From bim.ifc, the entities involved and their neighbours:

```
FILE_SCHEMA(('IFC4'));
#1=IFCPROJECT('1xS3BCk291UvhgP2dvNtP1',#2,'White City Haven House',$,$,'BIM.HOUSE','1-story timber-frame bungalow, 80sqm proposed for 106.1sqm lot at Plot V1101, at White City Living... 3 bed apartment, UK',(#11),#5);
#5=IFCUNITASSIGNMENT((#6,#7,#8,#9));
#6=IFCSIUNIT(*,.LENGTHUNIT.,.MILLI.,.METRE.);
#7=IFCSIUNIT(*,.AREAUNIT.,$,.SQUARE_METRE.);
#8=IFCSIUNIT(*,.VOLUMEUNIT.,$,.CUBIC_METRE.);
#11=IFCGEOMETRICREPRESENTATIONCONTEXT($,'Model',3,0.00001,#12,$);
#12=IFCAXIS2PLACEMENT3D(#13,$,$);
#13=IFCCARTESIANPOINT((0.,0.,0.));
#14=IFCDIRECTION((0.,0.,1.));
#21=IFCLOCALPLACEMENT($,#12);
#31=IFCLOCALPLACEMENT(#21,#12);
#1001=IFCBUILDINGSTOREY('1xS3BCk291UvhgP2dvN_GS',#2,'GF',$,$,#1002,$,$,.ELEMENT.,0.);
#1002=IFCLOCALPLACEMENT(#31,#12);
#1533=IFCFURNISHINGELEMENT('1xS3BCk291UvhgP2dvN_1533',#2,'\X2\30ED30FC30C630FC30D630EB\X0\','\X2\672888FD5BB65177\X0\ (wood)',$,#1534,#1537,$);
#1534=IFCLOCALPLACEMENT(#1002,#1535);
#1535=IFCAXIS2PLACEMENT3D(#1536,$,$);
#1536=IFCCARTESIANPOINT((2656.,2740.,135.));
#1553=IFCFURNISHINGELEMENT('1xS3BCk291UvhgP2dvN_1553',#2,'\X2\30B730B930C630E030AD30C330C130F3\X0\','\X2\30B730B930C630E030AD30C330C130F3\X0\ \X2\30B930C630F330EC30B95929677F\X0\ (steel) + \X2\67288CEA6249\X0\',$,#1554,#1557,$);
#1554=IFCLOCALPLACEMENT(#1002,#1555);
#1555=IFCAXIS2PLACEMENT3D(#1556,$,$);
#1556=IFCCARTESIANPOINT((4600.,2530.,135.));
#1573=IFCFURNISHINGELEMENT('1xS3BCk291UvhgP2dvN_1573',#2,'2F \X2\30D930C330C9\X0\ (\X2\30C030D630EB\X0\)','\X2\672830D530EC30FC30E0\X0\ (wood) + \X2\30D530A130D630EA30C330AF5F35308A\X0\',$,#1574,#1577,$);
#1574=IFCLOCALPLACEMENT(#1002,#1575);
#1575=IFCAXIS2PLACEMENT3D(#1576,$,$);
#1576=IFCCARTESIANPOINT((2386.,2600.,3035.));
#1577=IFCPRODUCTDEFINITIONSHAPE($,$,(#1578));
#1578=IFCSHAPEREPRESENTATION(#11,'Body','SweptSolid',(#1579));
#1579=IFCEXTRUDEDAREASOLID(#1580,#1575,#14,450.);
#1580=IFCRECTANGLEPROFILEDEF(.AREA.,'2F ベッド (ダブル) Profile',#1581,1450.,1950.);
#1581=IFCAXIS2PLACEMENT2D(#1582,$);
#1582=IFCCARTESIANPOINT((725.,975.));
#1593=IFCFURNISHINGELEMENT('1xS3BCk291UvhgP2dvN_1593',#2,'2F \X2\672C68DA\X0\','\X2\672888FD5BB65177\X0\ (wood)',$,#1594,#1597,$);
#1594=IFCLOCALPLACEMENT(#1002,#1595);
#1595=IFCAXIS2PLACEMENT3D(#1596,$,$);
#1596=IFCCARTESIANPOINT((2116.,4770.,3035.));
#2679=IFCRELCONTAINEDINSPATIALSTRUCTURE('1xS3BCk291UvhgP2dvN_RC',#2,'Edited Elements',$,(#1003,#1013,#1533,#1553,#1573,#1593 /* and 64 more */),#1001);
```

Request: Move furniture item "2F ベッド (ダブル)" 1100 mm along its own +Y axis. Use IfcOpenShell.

```python
import ifcopenshell
import ifcopenshell.api.geometry
import ifcopenshell.util.placement

model = ifcopenshell.open("bim.ifc")

item = model.by_guid("1xS3BCk291UvhgP2dvN_1573")
matrix = ifcopenshell.util.placement.get_local_placement(item.ObjectPlacement)
matrix[:3, 3] += matrix[:3, 1] * 1100.0
ifcopenshell.api.geometry.edit_object_placement(model, product=item, matrix=matrix, is_si=False)

print(ifcopenshell.util.placement.get_local_placement(item.ObjectPlacement).round(3) + 0.0)

model.write("bim-out.ifc")
```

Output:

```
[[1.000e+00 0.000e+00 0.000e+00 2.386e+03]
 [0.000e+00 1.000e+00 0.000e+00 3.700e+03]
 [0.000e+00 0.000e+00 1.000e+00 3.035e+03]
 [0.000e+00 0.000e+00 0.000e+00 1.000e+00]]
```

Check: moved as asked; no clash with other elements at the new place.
